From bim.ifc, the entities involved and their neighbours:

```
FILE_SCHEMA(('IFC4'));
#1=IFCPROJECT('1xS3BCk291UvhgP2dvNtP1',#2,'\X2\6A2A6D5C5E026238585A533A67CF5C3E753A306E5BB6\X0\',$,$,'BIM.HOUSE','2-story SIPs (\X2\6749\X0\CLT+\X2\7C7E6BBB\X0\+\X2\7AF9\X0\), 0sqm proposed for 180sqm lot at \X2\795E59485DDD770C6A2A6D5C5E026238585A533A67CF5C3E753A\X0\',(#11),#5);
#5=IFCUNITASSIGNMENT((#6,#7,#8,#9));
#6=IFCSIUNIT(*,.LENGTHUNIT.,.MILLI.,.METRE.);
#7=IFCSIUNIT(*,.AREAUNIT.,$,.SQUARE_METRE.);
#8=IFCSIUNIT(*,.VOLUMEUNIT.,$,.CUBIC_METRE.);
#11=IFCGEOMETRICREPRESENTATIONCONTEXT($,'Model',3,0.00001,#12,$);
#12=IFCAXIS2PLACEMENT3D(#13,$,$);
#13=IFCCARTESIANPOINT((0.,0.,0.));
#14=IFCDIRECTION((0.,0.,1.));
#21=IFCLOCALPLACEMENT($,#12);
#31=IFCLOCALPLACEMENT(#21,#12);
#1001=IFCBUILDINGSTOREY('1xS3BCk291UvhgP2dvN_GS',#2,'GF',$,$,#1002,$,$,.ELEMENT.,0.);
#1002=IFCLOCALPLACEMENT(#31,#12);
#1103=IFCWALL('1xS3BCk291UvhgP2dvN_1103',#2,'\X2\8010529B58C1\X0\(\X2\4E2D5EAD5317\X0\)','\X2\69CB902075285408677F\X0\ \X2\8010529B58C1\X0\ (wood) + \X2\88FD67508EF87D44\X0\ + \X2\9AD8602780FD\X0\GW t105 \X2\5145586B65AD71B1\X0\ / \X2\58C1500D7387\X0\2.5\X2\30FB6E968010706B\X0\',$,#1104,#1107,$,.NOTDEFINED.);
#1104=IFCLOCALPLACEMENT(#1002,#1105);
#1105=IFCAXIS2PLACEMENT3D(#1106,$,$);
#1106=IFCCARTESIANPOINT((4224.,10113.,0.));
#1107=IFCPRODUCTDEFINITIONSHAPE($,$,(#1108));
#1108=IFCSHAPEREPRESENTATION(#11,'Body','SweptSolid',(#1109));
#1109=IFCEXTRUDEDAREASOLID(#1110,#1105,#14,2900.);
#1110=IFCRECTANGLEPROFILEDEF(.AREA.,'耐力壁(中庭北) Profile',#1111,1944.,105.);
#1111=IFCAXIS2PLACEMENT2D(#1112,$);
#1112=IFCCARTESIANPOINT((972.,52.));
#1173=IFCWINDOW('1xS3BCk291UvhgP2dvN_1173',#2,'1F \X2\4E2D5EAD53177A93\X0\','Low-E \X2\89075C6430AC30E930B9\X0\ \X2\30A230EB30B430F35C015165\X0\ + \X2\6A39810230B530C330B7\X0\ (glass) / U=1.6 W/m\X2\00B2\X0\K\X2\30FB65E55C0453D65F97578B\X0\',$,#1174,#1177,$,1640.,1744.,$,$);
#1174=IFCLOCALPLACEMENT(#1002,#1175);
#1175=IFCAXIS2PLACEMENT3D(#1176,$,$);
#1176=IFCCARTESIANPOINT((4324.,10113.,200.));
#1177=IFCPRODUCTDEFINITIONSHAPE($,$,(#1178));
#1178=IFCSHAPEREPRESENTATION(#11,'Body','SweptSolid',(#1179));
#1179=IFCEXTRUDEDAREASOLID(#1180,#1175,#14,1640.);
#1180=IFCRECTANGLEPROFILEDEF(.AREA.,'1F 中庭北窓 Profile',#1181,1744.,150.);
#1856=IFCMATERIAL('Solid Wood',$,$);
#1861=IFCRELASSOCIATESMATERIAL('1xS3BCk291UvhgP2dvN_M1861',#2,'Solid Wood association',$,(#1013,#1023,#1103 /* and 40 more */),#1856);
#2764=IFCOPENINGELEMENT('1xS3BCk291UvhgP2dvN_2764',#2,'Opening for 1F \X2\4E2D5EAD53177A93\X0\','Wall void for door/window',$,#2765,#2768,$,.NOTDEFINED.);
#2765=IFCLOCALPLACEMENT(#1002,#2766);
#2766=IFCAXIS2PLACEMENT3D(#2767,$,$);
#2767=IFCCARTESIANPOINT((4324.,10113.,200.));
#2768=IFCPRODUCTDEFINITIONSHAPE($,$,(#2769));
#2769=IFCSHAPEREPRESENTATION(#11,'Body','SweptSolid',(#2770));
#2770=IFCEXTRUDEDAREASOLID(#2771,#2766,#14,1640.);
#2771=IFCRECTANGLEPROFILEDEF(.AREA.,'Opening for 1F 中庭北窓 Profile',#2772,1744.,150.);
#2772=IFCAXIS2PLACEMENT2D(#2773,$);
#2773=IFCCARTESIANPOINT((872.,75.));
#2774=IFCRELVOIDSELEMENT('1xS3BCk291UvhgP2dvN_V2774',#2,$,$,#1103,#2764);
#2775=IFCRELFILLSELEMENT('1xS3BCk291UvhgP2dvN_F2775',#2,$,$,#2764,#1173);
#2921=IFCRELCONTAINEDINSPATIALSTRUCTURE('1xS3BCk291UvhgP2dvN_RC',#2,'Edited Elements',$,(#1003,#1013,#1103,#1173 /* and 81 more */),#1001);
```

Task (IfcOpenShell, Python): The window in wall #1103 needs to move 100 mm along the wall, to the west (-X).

```python
import ifcopenshell
import ifcopenshell.api.geometry
import ifcopenshell.util.placement
import ifcopenshell.util.unit

model = ifcopenshell.open("bim.ifc")
unit_scale = ifcopenshell.util.unit.calculate_unit_scale(model)

window = model.by_id(1173)
opening = window.FillsVoids[0].RelatingOpeningElement
wall = opening.VoidsElements[0].RelatingBuildingElement

wall_matrix = ifcopenshell.util.placement.get_local_placement(wall.ObjectPlacement)
shift = wall_matrix[:3, 0] * -0.1 / unit_scale
before = ifcopenshell.util.placement.get_local_placement(window.ObjectPlacement)[:3, 3].copy()

# The window is not placed relative to its opening, so move both.
for product in (opening, window):
    matrix = ifcopenshell.util.placement.get_local_placement(product.ObjectPlacement)
    matrix[:3, 3] += shift
    ifcopenshell.api.geometry.edit_object_placement(model, product=product, matrix=matrix, is_si=False)

after = ifcopenshell.util.placement.get_local_placement(window.ObjectPlacement)[:3, 3]
print("window moved by", (after - before).round(3) + 0.0)

model.write("bim_v2.ifc")
```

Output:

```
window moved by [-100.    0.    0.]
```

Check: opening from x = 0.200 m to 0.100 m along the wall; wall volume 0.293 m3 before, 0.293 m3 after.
